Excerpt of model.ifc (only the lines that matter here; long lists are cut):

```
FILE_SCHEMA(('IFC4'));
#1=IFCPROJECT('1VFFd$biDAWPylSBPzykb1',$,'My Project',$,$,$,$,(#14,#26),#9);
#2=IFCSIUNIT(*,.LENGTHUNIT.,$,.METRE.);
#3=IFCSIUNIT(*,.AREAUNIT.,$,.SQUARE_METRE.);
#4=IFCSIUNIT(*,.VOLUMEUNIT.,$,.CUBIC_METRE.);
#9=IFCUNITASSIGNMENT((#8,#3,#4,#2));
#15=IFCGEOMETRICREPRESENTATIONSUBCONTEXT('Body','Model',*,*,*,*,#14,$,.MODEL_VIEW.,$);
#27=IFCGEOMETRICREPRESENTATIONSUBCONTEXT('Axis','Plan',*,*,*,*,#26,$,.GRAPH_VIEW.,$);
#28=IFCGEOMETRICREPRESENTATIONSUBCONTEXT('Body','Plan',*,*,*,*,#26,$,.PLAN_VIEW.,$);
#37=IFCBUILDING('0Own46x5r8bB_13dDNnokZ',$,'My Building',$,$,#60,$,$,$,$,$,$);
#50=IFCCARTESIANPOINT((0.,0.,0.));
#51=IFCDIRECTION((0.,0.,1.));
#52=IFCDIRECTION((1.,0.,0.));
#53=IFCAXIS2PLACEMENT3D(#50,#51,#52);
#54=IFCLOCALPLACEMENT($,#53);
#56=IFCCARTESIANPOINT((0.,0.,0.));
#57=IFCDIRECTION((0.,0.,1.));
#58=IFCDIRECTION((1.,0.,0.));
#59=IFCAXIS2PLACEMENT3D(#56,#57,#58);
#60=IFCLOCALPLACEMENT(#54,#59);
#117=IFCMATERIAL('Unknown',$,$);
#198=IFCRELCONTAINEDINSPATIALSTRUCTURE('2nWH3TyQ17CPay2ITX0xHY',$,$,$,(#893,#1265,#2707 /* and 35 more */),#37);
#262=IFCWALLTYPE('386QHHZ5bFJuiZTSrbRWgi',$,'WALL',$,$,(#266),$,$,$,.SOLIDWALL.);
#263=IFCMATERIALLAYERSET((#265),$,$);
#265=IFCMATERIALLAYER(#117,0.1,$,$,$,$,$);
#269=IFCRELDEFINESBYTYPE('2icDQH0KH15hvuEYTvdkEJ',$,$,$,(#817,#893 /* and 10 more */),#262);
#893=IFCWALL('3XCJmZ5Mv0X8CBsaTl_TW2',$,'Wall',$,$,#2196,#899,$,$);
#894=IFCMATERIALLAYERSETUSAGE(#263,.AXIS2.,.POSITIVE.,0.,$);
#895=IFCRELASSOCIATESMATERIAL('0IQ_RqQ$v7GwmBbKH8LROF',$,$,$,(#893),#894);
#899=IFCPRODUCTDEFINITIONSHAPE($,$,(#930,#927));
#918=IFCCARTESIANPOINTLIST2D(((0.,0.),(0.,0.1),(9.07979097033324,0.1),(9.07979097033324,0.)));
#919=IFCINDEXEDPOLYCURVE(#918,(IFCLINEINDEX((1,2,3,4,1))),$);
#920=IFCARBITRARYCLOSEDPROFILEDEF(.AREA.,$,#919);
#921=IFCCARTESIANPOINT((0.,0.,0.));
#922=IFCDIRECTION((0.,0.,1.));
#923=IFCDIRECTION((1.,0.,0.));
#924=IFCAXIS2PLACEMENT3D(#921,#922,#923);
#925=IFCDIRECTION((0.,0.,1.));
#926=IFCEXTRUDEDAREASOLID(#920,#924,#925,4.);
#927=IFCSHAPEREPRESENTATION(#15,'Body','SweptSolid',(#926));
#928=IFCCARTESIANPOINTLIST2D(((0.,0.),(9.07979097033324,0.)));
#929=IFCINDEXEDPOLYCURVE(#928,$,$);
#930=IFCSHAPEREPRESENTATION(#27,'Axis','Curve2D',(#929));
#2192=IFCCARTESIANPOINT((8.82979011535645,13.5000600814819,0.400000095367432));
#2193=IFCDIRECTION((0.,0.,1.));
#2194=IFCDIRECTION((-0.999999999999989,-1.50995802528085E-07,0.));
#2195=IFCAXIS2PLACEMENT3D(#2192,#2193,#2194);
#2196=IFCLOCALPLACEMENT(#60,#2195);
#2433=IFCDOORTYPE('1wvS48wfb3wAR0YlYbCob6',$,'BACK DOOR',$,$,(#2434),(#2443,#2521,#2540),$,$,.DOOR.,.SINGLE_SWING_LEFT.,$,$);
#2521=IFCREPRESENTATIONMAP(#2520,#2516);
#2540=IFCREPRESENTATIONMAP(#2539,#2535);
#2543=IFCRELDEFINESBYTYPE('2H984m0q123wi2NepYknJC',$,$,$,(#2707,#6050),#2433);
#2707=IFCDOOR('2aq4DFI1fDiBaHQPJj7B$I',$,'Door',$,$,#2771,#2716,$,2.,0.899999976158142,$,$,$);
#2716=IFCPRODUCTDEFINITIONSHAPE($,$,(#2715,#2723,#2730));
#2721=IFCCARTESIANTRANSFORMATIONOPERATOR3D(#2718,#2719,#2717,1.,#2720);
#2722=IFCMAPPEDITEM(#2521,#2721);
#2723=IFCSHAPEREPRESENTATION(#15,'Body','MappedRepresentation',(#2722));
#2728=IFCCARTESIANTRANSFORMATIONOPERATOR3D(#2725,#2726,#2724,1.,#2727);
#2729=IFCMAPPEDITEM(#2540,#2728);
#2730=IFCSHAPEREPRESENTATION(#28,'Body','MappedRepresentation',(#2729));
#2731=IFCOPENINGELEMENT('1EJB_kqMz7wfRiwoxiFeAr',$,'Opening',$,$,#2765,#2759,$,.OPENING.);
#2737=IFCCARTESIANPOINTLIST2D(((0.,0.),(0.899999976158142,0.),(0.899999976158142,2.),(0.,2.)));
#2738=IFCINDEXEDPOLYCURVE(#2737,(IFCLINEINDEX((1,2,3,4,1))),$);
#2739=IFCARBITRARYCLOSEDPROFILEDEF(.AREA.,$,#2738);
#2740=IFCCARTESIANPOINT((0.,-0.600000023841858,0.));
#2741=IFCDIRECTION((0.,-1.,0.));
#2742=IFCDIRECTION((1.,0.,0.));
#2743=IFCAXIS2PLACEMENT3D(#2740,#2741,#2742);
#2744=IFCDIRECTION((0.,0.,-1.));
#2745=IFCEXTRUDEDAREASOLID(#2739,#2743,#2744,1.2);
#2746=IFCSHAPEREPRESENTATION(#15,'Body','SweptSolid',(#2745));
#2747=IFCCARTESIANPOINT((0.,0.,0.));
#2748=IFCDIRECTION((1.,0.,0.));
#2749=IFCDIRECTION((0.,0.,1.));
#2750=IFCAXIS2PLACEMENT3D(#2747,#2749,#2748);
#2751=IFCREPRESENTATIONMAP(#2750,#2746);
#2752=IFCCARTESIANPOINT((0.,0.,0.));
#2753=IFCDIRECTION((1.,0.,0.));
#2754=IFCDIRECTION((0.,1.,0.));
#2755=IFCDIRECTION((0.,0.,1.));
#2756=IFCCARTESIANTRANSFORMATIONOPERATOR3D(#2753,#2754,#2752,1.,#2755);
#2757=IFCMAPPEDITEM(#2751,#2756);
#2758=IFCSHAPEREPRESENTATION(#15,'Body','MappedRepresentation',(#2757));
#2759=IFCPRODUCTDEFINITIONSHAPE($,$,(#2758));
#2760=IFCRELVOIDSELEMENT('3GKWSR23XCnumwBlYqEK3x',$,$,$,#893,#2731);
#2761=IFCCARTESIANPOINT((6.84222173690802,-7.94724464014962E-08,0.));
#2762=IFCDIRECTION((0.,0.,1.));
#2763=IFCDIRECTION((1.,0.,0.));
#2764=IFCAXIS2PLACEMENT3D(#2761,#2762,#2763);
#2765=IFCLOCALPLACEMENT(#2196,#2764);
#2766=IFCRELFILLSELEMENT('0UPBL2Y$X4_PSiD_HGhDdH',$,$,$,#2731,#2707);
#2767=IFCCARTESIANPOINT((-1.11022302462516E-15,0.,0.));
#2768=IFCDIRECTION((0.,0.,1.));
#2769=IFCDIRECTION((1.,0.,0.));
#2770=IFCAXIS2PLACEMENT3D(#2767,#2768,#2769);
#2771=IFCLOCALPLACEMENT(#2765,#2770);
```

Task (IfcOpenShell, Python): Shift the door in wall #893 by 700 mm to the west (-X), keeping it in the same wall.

```python
import ifcopenshell
import ifcopenshell.api.geometry
import ifcopenshell.util.placement
import ifcopenshell.util.unit

model = ifcopenshell.open("model.ifc")
unit_scale = ifcopenshell.util.unit.calculate_unit_scale(model)

door = model.by_guid("2aq4DFI1fDiBaHQPJj7B$I")
opening = door.FillsVoids[0].RelatingOpeningElement
wall = opening.VoidsElements[0].RelatingBuildingElement

wall_matrix = ifcopenshell.util.placement.get_local_placement(wall.ObjectPlacement)
shift = wall_matrix[:3, 0] * 0.7 / unit_scale
before = ifcopenshell.util.placement.get_local_placement(door.ObjectPlacement)[:3, 3].copy()

# The door is placed relative to its opening, so it follows when the opening moves.
matrix = ifcopenshell.util.placement.get_local_placement(opening.ObjectPlacement)
matrix[:3, 3] += shift
ifcopenshell.api.geometry.edit_object_placement(
    model, product=opening, matrix=matrix, is_si=False, should_transform_children=True
)

after = ifcopenshell.util.placement.get_local_placement(door.ObjectPlacement)[:3, 3]
print("door moved by", (after - before).round(3) + 0.0)

model.write("model_rev.ifc")
```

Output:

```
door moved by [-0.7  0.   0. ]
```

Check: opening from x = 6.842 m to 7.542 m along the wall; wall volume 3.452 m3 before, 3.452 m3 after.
